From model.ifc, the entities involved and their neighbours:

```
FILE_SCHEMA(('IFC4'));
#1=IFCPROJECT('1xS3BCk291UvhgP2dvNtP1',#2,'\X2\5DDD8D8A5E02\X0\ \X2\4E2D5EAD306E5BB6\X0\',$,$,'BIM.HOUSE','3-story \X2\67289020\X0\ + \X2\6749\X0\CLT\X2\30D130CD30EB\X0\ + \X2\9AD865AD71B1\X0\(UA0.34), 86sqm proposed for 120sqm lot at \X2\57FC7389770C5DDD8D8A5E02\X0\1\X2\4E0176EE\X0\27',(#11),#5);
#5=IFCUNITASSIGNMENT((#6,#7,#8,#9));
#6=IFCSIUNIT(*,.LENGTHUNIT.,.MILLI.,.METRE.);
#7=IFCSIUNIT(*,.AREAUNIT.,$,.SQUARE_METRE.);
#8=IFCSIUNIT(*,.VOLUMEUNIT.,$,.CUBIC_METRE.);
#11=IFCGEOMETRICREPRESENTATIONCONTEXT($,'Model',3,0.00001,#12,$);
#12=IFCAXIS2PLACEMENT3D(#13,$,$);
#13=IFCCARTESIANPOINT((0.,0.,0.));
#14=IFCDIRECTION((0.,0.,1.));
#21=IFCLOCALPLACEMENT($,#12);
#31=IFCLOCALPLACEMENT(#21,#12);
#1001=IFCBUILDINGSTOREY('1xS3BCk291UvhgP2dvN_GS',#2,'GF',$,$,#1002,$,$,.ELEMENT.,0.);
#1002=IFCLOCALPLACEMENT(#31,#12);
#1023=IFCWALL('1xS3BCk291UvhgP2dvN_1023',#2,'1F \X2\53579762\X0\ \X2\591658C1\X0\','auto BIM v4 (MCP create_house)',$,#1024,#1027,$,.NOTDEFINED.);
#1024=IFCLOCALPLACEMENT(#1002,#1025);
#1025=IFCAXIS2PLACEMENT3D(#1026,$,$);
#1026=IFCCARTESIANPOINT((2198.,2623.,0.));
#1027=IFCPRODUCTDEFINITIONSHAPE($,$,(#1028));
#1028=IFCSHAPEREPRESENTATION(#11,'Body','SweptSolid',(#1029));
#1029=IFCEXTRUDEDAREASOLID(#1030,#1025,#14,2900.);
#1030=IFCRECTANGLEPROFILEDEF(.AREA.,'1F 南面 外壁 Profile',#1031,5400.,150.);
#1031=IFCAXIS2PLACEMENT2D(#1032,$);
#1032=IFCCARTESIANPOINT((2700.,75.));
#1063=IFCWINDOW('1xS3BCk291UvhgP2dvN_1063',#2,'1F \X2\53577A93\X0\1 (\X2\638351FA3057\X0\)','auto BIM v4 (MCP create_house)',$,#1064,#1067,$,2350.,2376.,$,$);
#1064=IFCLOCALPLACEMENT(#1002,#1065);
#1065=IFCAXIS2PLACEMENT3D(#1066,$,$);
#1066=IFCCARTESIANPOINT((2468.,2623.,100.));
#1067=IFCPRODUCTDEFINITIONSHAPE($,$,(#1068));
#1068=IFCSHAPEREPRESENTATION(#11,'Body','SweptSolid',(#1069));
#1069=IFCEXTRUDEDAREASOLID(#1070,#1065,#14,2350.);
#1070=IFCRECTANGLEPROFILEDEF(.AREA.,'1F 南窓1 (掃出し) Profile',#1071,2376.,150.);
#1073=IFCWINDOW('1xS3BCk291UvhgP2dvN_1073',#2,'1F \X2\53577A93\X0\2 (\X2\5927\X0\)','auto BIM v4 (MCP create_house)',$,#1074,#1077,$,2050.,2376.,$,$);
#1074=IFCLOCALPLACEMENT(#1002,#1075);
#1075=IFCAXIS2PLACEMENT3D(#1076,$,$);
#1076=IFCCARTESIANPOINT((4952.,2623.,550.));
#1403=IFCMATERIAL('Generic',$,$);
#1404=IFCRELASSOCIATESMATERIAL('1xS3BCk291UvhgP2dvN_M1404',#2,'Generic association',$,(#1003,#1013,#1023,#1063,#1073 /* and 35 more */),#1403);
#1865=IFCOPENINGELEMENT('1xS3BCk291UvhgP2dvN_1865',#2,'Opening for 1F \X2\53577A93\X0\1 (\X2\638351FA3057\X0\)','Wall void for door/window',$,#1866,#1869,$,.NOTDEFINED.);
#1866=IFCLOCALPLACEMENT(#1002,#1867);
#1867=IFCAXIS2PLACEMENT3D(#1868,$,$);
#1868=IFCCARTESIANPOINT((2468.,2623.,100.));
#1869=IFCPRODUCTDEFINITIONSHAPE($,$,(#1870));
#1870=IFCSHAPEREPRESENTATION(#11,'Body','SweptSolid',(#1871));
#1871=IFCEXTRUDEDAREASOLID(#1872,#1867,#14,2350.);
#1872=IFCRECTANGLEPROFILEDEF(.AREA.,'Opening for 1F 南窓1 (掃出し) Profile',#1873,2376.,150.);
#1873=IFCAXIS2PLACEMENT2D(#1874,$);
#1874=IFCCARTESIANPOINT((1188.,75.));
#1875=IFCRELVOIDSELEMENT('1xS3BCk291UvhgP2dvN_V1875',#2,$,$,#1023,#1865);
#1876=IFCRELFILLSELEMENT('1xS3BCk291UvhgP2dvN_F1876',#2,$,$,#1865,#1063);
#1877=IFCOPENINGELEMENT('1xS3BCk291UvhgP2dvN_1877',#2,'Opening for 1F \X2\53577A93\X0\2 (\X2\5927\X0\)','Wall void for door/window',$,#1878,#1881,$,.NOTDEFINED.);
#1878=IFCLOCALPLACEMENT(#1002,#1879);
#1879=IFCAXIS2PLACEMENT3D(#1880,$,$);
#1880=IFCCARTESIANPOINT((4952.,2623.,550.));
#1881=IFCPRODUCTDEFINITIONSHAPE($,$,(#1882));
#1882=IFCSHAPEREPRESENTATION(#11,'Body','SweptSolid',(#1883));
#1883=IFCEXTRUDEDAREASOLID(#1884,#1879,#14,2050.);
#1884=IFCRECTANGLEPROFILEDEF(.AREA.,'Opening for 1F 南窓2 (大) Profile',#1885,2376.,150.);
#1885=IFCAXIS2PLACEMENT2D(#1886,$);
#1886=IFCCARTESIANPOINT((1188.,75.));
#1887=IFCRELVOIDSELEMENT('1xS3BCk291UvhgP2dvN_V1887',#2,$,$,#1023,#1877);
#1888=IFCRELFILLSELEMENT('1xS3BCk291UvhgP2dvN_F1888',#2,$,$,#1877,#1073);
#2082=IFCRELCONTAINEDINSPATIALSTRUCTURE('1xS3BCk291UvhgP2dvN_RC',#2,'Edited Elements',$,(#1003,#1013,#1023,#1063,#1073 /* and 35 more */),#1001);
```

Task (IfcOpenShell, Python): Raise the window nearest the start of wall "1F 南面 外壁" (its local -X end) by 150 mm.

```python
import numpy as np
import ifcopenshell
import ifcopenshell.api.geometry
import ifcopenshell.util.placement
import ifcopenshell.util.unit

model = ifcopenshell.open("model.ifc")
unit_scale = ifcopenshell.util.unit.calculate_unit_scale(model)

window = model.by_guid("1xS3BCk291UvhgP2dvN_1063")
opening = window.FillsVoids[0].RelatingOpeningElement
dz = 150.0

shift = np.array([0.0, 0.0, dz])
# The window is not placed relative to its opening, so move both.
for product in (opening, window):
    matrix = ifcopenshell.util.placement.get_local_placement(product.ObjectPlacement)
    matrix[:3, 3] += shift
    ifcopenshell.api.geometry.edit_object_placement(model, product=product, matrix=matrix, is_si=False)

print(f"moved by {dz * unit_scale:+.3f} m")

model.write("model_rev.ifc")
```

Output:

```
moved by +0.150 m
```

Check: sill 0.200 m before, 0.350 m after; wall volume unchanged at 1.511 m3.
